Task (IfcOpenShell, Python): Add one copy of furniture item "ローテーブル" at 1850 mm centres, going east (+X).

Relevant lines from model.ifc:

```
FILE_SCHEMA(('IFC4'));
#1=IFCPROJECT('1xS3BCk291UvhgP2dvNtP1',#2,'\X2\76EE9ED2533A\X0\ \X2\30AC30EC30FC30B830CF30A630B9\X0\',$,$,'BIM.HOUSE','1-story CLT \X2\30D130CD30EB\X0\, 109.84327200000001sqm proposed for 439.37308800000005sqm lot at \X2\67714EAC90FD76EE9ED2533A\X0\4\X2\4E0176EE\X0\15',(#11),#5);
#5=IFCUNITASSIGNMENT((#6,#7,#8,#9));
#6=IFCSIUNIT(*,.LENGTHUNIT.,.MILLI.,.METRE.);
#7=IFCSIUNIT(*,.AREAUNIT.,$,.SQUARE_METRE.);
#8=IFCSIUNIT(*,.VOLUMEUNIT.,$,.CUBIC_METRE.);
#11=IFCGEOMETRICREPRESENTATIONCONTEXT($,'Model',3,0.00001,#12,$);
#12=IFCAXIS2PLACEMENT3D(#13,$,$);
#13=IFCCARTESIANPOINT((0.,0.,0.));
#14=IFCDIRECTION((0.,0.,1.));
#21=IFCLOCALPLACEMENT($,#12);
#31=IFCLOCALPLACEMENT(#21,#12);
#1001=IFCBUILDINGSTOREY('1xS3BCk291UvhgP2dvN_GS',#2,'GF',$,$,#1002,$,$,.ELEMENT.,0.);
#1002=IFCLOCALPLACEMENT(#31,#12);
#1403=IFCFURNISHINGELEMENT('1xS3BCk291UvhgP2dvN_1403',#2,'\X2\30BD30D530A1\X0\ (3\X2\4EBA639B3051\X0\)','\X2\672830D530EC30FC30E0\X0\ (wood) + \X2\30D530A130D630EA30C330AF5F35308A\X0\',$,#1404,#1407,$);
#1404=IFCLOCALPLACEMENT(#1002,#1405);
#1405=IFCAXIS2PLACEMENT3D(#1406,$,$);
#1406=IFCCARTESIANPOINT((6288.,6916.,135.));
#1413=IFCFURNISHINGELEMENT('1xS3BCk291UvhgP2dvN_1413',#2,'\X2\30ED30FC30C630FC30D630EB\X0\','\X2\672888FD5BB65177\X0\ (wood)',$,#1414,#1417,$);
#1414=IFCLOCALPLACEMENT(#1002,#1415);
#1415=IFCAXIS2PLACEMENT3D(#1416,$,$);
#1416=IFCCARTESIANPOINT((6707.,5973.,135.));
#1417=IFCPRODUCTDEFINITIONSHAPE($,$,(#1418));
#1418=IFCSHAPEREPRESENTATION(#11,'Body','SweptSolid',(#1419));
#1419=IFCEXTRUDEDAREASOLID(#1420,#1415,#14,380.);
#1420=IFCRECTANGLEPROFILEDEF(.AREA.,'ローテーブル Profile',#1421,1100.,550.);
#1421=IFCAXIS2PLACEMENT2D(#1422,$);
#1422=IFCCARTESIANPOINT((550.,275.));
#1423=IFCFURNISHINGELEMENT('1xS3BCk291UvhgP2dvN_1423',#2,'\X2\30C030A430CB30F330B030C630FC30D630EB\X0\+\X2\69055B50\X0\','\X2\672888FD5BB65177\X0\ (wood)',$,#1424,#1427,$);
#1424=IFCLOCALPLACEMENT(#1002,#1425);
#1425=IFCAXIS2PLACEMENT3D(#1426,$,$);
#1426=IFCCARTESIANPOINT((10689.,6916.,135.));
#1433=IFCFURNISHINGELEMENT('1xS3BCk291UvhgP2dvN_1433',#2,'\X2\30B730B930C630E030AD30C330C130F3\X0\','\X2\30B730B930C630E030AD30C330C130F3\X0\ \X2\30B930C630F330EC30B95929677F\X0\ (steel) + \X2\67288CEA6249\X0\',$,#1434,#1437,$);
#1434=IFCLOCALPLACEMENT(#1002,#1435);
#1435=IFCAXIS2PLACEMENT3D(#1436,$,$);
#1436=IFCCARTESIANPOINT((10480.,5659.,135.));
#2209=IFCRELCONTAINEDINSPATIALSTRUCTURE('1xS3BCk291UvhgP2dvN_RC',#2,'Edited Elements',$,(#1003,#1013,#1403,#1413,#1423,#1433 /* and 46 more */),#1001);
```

```python
import numpy as np
import ifcopenshell
import ifcopenshell.api.geometry
import ifcopenshell.api.root
import ifcopenshell.util.element
import ifcopenshell.util.placement
import ifcopenshell.util.unit

model = ifcopenshell.open("model.ifc")
unit_scale = ifcopenshell.util.unit.calculate_unit_scale(model)


def reuse_history(source, copy):
    """copy_class also copies each property set's owner history, people and application; keep the originals."""
    for rel in copy.IsDefinedBy:
        if rel.is_a("IfcRelDefinesByProperties") and (history := rel.RelatingPropertyDefinition.OwnerHistory):
            rel.RelatingPropertyDefinition.OwnerHistory = source.OwnerHistory
            ifcopenshell.util.element.remove_deep2(model, history)


source = model.by_guid("1xS3BCk291UvhgP2dvN_1413")
base = ifcopenshell.util.placement.get_local_placement(source.ObjectPlacement)
step = np.array([1.0, 0.0, 0.0]) * 1.85 / unit_scale

for i in range(1, 2):
    copy = ifcopenshell.api.root.copy_class(model, product=source)
    copy.Representation = ifcopenshell.util.element.copy_deep(
        model, source.Representation, exclude=["IfcGeometricRepresentationContext", "IfcRepresentationMap"]
    )
    reuse_history(source, copy)
    matrix = base.copy()
    matrix[:3, 3] += i * step
    print("added at", matrix[:3, 3].round(3) + 0.0)
    ifcopenshell.api.geometry.edit_object_placement(model, product=copy, matrix=matrix, is_si=False)

model.write("model_v2.ifc")
```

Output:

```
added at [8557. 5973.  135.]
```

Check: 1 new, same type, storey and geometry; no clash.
